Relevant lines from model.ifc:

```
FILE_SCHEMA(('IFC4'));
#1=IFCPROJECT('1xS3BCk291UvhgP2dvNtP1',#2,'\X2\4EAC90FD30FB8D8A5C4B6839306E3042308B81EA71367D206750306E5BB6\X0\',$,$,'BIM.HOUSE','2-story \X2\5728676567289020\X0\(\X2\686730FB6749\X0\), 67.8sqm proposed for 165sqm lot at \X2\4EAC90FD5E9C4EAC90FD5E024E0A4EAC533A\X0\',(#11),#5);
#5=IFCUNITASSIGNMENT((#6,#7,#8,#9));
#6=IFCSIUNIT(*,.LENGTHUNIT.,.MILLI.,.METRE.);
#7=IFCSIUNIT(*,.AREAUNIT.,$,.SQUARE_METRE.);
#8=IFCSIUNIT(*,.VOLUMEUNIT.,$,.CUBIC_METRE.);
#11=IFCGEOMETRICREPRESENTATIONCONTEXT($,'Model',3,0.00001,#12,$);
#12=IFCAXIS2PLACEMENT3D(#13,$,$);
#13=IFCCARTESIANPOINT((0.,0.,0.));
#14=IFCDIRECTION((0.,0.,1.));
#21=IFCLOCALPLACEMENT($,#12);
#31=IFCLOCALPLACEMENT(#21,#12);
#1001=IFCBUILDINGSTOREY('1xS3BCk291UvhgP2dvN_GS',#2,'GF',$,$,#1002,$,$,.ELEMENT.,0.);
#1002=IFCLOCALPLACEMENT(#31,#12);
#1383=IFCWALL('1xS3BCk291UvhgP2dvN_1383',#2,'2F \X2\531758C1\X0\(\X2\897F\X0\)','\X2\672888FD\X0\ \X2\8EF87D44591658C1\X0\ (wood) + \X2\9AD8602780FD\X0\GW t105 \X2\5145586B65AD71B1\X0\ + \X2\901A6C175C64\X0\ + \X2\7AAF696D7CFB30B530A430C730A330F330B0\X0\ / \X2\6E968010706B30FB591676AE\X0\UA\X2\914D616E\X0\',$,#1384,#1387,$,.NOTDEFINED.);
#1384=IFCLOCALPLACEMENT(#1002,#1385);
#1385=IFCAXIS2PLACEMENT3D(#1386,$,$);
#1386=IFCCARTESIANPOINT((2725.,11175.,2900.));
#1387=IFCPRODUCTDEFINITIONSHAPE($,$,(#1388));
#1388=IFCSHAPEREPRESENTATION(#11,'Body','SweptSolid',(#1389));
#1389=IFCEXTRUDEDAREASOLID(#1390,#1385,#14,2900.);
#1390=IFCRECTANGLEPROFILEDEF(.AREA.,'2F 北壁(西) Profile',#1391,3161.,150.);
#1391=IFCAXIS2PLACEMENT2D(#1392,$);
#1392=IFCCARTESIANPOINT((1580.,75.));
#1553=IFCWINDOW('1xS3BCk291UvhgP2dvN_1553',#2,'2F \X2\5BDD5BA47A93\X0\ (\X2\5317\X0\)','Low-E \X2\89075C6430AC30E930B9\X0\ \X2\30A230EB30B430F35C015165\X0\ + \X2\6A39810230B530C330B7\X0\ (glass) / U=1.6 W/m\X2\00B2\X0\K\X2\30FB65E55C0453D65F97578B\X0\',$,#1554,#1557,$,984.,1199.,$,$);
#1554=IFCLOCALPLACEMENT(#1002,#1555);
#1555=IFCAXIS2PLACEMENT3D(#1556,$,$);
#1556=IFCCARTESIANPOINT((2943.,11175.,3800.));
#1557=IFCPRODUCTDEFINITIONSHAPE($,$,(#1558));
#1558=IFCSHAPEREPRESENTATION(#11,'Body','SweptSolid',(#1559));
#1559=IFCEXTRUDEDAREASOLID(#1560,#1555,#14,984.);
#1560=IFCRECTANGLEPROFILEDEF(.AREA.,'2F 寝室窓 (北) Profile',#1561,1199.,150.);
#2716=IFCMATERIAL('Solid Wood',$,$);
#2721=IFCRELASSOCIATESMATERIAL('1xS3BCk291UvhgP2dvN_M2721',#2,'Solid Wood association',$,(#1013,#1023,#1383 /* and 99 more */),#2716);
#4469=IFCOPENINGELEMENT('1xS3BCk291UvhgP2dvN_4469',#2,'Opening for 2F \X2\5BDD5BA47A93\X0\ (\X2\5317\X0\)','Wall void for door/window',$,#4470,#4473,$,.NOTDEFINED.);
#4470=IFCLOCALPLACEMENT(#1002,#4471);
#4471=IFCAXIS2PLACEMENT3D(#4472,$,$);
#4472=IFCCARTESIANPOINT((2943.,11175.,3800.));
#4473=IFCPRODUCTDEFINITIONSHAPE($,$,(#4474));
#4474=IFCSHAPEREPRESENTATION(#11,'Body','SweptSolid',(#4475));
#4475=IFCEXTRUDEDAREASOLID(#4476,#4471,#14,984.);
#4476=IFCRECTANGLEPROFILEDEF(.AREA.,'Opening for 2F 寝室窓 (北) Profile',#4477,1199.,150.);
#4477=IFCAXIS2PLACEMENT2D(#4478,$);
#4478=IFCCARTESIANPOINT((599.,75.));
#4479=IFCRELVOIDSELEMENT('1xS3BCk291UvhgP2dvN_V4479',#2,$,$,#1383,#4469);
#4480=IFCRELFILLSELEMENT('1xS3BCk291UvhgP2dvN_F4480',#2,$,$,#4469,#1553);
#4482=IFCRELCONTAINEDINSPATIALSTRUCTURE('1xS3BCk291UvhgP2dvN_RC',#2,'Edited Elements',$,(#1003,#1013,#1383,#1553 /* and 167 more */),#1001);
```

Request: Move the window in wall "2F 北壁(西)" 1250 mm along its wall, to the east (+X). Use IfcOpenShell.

```python
import ifcopenshell
import ifcopenshell.api.geometry
import ifcopenshell.util.placement

model = ifcopenshell.open("model.ifc")

window = model.by_id(1553)
opening = window.FillsVoids[0].RelatingOpeningElement
wall = opening.VoidsElements[0].RelatingBuildingElement

wall_matrix = ifcopenshell.util.placement.get_local_placement(wall.ObjectPlacement)
shift = wall_matrix[:3, 0] * 1250.0
before = ifcopenshell.util.placement.get_local_placement(window.ObjectPlacement)[:3, 3].copy()

# The window is not placed relative to its opening, so move both.
for product in (opening, window):
    matrix = ifcopenshell.util.placement.get_local_placement(product.ObjectPlacement)
    matrix[:3, 3] += shift
    ifcopenshell.api.geometry.edit_object_placement(model, product=product, matrix=matrix, is_si=False)

after = ifcopenshell.util.placement.get_local_placement(window.ObjectPlacement)[:3, 3]
print("window moved by", (after - before).round(3) + 0.0)

model.write("model_updated.ifc")
```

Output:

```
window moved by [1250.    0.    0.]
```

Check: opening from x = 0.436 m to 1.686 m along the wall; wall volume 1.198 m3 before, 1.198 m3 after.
